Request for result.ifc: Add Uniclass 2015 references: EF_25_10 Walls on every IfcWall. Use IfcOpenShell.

First a look at what the model holds.

```python
import ifcopenshell

model = ifcopenshell.open("result.ifc")
print(model.schema)
print("classifications:", [c.Name for c in model.by_type("IfcClassification")])
for ifc_class in ("IfcDoor", "IfcRoof", "IfcStair", "IfcWall", "IfcWindow"):
    print(ifc_class, len(model.by_type(ifc_class)))
```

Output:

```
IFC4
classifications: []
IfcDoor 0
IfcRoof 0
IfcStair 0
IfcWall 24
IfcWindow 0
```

```python
import ifcopenshell
import ifcopenshell.api.classification

model = ifcopenshell.open("result.ifc")

system = ifcopenshell.api.classification.add_classification(model, classification="Uniclass 2015")

codes = {
    "IfcWall": ("EF_25_10", "Walls"),
}
for ifc_class, (code, name) in codes.items():
    products = model.by_type(ifc_class)
    ifcopenshell.api.classification.add_reference(
        model, products=products, classification=system, identification=code, name=name
    )
    print(code, len(products))

model.write("result_rev.ifc")
```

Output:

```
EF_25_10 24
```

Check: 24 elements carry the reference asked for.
